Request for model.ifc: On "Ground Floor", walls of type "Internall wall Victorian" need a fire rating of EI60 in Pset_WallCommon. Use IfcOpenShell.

First a look at what the model holds.

```python
import ifcopenshell
import ifcopenshell.util.element

model = ifcopenshell.open("model.ifc")
print(model.schema)
storey = next(s for s in model.by_type("IfcBuildingStorey") if s.Name == "Ground Floor")
walls = [e for e in ifcopenshell.util.element.get_decomposition(storey) if e.is_a("IfcWall")]
seen = {}
for e in walls:
    element_type = ifcopenshell.util.element.get_type(e)
    key = (element_type.Name if element_type != e and element_type else None, ifcopenshell.util.element.get_pset(e, "Pset_WallCommon", "FireRating"))
    seen[key] = seen.get(key, 0) + 1
for (name, value), count in sorted(seen.items(), key=str):
    print(count, "x", name, "|", value)
```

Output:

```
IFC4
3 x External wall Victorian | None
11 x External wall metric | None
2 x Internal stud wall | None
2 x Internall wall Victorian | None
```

```python
import ifcopenshell
import ifcopenshell.api.pset
import ifcopenshell.util.element

model = ifcopenshell.open("model.ifc")

storey = next(s for s in model.by_type("IfcBuildingStorey") if s.Name == "Ground Floor")
walls = [e for e in ifcopenshell.util.element.get_decomposition(storey) if e.is_a("IfcWall")]

count = 0
for e in walls:
    element_type = ifcopenshell.util.element.get_type(e)
    if element_type in (None, e) or element_type.Name != "Internall wall Victorian":
        continue
    # add_pset returns the element's existing set when there is one.
    pset = ifcopenshell.api.pset.add_pset(model, product=e, name="Pset_WallCommon")
    ifcopenshell.api.pset.edit_pset(model, pset=pset, properties={"FireRating": "EI60"})
    count += 1

print(count, "walls updated")

model.write("model-out.ifc")
```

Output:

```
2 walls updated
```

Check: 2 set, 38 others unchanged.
